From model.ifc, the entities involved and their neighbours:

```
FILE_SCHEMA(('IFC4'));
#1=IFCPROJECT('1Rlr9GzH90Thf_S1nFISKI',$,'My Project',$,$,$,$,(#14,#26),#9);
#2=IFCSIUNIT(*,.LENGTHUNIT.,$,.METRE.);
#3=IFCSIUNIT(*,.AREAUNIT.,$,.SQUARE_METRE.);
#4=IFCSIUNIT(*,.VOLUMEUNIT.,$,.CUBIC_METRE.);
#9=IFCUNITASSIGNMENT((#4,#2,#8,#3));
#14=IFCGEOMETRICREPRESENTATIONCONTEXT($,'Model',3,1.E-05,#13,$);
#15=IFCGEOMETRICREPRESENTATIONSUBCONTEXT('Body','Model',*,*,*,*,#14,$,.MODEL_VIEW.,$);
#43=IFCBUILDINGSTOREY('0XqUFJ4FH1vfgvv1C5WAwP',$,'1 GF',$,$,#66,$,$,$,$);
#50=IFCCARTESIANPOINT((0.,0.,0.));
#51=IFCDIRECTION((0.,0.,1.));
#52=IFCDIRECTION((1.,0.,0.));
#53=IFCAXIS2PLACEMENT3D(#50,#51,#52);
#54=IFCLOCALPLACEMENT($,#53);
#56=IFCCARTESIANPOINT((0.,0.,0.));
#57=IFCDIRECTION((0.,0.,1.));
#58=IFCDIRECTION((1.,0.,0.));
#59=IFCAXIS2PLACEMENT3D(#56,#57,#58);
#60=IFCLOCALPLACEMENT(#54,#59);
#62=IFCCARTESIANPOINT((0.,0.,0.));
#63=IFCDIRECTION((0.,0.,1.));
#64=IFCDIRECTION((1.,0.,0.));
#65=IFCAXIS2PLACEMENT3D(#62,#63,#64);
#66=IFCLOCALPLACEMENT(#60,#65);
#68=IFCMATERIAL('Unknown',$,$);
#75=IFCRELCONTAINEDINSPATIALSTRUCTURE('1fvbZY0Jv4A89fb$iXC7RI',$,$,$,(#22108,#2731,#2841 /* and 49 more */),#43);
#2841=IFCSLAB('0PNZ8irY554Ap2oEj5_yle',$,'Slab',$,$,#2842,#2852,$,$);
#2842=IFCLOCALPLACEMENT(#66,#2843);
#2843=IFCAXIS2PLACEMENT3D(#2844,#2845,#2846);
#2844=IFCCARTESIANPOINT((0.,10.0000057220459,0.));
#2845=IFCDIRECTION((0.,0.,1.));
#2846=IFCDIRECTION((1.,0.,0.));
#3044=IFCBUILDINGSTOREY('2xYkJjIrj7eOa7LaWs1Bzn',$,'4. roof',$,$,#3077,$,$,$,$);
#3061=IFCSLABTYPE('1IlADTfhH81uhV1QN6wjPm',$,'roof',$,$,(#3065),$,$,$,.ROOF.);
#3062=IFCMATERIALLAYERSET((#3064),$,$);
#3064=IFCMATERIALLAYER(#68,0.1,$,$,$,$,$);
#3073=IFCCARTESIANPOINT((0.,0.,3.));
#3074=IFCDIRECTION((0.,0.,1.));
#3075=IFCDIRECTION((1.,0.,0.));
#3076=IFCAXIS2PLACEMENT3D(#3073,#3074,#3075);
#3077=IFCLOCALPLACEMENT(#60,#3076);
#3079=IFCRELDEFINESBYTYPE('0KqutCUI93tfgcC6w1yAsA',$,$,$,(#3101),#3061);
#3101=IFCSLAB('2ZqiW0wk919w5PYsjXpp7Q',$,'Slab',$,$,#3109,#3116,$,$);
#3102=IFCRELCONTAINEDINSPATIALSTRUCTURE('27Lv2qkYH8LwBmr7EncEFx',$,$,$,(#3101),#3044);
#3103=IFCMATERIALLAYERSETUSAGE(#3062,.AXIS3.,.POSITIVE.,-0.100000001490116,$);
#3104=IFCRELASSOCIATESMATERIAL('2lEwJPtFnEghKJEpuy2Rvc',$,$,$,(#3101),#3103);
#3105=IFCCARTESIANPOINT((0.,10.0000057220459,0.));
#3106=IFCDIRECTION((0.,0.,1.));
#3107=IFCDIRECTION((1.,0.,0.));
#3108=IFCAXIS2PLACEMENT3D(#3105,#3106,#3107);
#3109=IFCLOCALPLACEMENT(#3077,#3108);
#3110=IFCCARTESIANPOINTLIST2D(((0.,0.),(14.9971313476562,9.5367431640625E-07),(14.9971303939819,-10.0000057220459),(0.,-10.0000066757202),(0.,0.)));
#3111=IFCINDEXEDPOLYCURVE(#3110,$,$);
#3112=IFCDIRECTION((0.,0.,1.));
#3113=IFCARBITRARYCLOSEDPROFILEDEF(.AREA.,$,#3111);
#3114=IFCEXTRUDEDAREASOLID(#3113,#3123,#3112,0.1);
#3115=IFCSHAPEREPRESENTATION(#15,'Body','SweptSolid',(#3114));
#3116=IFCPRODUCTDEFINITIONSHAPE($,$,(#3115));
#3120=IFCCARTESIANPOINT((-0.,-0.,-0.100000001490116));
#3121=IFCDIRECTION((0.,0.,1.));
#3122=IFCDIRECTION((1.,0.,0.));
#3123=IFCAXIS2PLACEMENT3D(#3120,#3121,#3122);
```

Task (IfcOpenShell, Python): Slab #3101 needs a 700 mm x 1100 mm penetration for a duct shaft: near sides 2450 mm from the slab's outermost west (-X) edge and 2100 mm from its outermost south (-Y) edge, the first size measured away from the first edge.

```python
import numpy as np
import ifcopenshell
import ifcopenshell.api.feature
import ifcopenshell.api.geometry
import ifcopenshell.api.root
import ifcopenshell.geom
import ifcopenshell.util.placement
import ifcopenshell.util.representation
import ifcopenshell.util.shape
import ifcopenshell.util.unit

model = ifcopenshell.open("model.ifc")
unit_scale = ifcopenshell.util.unit.calculate_unit_scale(model)
settings = ifcopenshell.geom.settings()


def volume(element):
    """Net volume in cubic metres, openings subtracted."""
    shape = ifcopenshell.geom.create_shape(settings, element)
    return ifcopenshell.util.shape.get_volume(shape.geometry)


slab = model.by_id(3101)
before = volume(slab)

# Extent in the slab's own axes, in metres. The edges named are its -X and -Y sides.
slab_shape = ifcopenshell.geom.create_shape(settings, slab)
vertices = ifcopenshell.util.shape.get_vertices(slab_shape.geometry)
x_min, y_min, bottom = vertices.min(axis=0)
top = vertices[:, 2].max()

opening = ifcopenshell.api.root.create_entity(model, ifc_class="IfcOpeningElement", name="Duct shaft opening", predefined_type="OPENING")
context = ifcopenshell.util.representation.get_context(model, "Model", "Body", "MODEL_VIEW")
width, depth = 0.7, 1.1
outline = [(0.0, 0.0), (width, 0.0), (width, depth), (0.0, depth), (0.0, 0.0)]
# Overshoot both faces by 50 mm so the cut is clean.
shape = ifcopenshell.api.geometry.add_slab_representation(
    model, context=context, depth=top - bottom + 0.1, polyline=outline
)
ifcopenshell.api.geometry.assign_representation(model, product=opening, representation=shape)

matrix = ifcopenshell.util.placement.get_local_placement(slab.ObjectPlacement)
matrix[:, 3] = matrix @ np.append(np.array([x_min + 2.45, y_min + 2.1, bottom - 0.05]) / unit_scale, 1.0)
ifcopenshell.api.geometry.edit_object_placement(model, product=opening, matrix=matrix, is_si=False)
ifcopenshell.api.feature.add_feature(model, feature=opening, element=slab)

after = volume(slab)

print(f"slab volume {before:.3f} -> {after:.3f} m3")

model.write("model_updated.ifc")
```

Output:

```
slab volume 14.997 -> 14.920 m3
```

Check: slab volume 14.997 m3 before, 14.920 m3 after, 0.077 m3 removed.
